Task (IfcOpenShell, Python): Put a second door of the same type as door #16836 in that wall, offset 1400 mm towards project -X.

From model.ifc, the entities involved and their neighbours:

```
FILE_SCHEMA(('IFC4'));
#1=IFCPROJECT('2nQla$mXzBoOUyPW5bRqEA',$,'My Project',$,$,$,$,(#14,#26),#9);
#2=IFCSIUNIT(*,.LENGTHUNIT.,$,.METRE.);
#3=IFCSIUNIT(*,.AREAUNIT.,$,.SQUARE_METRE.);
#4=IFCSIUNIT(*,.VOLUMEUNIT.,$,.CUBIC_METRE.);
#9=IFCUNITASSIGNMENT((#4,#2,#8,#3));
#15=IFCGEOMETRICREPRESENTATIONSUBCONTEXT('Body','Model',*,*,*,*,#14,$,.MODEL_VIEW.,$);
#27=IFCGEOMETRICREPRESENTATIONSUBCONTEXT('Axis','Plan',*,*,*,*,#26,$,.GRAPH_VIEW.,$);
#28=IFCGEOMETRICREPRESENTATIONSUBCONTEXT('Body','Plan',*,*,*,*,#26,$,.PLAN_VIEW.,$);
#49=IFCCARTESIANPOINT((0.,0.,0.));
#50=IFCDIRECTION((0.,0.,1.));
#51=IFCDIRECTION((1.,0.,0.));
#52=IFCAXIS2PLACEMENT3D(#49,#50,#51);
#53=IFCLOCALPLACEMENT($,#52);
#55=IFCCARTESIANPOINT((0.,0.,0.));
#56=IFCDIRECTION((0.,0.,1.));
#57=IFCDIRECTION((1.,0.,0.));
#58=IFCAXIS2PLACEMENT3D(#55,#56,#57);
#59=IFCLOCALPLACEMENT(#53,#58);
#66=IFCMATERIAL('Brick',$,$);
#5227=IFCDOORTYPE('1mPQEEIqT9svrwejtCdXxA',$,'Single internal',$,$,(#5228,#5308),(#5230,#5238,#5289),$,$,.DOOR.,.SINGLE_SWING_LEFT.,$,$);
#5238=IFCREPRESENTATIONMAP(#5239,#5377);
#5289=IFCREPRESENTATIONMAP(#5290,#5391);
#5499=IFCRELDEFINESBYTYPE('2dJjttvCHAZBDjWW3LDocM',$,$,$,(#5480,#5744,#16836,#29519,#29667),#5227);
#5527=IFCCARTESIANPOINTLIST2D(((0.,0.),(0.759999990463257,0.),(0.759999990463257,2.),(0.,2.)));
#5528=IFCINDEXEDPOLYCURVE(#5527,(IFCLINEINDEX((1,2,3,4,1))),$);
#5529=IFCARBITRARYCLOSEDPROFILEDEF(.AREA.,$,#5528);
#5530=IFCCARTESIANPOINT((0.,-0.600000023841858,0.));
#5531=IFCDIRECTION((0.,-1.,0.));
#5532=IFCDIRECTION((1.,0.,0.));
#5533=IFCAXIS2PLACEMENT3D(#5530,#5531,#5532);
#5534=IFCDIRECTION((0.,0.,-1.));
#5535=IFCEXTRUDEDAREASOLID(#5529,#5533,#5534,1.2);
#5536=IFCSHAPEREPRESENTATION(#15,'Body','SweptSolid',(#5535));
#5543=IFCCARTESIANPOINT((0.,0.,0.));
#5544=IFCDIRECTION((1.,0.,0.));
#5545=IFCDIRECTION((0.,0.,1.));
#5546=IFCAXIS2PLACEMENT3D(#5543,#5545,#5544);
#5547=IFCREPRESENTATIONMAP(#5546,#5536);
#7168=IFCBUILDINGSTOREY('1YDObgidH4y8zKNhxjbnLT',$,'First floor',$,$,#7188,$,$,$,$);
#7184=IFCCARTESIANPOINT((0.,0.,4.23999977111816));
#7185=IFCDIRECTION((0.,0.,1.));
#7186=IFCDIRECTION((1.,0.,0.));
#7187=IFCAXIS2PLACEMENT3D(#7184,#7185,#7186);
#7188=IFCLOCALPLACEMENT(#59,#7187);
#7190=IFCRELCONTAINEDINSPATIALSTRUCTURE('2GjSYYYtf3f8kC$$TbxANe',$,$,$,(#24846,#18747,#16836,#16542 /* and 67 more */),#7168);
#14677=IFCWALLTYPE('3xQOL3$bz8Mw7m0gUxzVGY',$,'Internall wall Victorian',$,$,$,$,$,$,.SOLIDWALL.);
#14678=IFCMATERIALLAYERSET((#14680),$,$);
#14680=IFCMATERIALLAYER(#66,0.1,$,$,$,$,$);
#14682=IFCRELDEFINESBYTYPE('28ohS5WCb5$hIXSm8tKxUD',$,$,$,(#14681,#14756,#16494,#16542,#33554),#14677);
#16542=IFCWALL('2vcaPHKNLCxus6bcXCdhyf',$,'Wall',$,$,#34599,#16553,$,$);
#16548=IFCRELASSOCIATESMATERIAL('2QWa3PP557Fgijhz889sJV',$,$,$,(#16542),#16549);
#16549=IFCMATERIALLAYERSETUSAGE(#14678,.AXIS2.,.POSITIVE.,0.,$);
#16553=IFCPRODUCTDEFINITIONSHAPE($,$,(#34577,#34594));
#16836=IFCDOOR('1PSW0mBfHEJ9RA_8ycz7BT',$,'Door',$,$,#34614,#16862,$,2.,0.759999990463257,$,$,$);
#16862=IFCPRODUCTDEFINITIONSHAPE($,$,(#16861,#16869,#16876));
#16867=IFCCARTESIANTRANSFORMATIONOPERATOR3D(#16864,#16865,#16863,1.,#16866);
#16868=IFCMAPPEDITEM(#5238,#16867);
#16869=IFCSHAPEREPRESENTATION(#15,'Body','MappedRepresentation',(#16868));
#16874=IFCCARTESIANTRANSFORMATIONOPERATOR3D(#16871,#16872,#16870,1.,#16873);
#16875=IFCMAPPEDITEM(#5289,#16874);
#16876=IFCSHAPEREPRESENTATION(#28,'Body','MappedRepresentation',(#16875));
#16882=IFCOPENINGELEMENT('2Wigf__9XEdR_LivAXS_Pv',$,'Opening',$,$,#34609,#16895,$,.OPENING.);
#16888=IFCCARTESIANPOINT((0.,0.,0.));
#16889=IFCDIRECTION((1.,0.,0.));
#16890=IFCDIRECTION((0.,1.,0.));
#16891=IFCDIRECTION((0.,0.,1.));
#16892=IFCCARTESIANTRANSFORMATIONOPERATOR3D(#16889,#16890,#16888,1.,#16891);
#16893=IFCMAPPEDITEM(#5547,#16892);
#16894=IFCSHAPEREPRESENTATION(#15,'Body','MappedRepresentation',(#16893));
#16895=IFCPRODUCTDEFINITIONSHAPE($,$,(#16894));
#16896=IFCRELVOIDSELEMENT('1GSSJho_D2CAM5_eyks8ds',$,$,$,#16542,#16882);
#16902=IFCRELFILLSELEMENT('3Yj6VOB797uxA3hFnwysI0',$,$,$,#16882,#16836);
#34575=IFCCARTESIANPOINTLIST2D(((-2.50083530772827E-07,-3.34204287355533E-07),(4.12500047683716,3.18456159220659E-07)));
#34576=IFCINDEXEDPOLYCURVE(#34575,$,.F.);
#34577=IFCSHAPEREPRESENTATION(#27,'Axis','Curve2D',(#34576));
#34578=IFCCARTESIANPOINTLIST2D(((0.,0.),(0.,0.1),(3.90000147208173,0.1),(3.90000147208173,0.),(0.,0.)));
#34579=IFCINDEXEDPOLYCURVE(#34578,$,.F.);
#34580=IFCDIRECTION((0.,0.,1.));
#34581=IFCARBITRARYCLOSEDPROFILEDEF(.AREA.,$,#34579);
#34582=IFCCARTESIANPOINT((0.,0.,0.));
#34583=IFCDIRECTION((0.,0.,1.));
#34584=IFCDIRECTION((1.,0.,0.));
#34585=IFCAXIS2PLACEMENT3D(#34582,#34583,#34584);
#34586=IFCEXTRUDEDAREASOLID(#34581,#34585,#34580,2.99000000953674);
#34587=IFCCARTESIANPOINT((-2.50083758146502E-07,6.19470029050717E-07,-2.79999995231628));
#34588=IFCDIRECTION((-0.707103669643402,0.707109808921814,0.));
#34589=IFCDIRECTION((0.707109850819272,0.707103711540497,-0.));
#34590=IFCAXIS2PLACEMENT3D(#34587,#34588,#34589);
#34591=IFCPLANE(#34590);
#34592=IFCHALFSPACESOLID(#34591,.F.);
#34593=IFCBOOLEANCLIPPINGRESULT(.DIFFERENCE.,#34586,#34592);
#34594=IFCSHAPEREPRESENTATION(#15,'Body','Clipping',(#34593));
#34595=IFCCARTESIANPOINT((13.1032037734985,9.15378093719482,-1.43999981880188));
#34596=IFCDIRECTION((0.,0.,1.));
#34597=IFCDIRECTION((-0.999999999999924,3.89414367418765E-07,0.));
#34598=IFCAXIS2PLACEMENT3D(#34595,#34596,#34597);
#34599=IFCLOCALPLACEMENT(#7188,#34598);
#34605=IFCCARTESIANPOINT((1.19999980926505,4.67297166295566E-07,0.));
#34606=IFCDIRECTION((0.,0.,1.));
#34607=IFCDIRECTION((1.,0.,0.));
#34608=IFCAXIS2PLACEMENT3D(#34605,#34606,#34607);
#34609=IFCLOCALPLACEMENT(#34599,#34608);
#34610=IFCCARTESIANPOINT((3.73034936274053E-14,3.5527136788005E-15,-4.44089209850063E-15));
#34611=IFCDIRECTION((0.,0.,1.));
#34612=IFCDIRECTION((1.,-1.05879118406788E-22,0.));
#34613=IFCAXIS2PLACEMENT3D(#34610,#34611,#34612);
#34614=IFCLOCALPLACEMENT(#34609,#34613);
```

```python
import ifcopenshell
import ifcopenshell.api.feature
import ifcopenshell.api.geometry
import ifcopenshell.api.root
import ifcopenshell.geom
import ifcopenshell.util.element
import ifcopenshell.util.placement
import ifcopenshell.util.shape

model = ifcopenshell.open("model.ifc")
settings = ifcopenshell.geom.settings()


def volume(element):
    """Net volume in cubic metres, openings subtracted."""
    shape = ifcopenshell.geom.create_shape(settings, element)
    return ifcopenshell.util.shape.get_volume(shape.geometry)


door = model.by_id(16836)
opening = door.FillsVoids[0].RelatingOpeningElement
wall = opening.VoidsElements[0].RelatingBuildingElement
before = volume(wall)
shift = ifcopenshell.util.placement.get_local_placement(wall.ObjectPlacement)[:3, 0] * 1.4

# copy_class copies the void relationship, type, container and properties, but no geometry.
new_opening = ifcopenshell.api.root.copy_class(model, product=opening)
new_opening.Representation = ifcopenshell.util.element.copy_deep(
    model, opening.Representation, exclude=["IfcGeometricRepresentationContext", "IfcRepresentationMap"]
)
new_door = ifcopenshell.api.root.copy_class(model, product=door)
new_door.Representation = ifcopenshell.util.element.copy_deep(
    model, door.Representation, exclude=["IfcGeometricRepresentationContext", "IfcRepresentationMap"]
)
ifcopenshell.api.feature.add_filling(model, opening=new_opening, element=new_door)

for old, new in ((opening, new_opening), (door, new_door)):
    matrix = ifcopenshell.util.placement.get_local_placement(old.ObjectPlacement)
    matrix[:3, 3] += shift
    ifcopenshell.api.geometry.edit_object_placement(model, product=new, matrix=matrix, is_si=False)

after = volume(wall)

print(f"wall volume {before:.3f} -> {after:.3f} m3")

model.write("model_edited.ifc")
```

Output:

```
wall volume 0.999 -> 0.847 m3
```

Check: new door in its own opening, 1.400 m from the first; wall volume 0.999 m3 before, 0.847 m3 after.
